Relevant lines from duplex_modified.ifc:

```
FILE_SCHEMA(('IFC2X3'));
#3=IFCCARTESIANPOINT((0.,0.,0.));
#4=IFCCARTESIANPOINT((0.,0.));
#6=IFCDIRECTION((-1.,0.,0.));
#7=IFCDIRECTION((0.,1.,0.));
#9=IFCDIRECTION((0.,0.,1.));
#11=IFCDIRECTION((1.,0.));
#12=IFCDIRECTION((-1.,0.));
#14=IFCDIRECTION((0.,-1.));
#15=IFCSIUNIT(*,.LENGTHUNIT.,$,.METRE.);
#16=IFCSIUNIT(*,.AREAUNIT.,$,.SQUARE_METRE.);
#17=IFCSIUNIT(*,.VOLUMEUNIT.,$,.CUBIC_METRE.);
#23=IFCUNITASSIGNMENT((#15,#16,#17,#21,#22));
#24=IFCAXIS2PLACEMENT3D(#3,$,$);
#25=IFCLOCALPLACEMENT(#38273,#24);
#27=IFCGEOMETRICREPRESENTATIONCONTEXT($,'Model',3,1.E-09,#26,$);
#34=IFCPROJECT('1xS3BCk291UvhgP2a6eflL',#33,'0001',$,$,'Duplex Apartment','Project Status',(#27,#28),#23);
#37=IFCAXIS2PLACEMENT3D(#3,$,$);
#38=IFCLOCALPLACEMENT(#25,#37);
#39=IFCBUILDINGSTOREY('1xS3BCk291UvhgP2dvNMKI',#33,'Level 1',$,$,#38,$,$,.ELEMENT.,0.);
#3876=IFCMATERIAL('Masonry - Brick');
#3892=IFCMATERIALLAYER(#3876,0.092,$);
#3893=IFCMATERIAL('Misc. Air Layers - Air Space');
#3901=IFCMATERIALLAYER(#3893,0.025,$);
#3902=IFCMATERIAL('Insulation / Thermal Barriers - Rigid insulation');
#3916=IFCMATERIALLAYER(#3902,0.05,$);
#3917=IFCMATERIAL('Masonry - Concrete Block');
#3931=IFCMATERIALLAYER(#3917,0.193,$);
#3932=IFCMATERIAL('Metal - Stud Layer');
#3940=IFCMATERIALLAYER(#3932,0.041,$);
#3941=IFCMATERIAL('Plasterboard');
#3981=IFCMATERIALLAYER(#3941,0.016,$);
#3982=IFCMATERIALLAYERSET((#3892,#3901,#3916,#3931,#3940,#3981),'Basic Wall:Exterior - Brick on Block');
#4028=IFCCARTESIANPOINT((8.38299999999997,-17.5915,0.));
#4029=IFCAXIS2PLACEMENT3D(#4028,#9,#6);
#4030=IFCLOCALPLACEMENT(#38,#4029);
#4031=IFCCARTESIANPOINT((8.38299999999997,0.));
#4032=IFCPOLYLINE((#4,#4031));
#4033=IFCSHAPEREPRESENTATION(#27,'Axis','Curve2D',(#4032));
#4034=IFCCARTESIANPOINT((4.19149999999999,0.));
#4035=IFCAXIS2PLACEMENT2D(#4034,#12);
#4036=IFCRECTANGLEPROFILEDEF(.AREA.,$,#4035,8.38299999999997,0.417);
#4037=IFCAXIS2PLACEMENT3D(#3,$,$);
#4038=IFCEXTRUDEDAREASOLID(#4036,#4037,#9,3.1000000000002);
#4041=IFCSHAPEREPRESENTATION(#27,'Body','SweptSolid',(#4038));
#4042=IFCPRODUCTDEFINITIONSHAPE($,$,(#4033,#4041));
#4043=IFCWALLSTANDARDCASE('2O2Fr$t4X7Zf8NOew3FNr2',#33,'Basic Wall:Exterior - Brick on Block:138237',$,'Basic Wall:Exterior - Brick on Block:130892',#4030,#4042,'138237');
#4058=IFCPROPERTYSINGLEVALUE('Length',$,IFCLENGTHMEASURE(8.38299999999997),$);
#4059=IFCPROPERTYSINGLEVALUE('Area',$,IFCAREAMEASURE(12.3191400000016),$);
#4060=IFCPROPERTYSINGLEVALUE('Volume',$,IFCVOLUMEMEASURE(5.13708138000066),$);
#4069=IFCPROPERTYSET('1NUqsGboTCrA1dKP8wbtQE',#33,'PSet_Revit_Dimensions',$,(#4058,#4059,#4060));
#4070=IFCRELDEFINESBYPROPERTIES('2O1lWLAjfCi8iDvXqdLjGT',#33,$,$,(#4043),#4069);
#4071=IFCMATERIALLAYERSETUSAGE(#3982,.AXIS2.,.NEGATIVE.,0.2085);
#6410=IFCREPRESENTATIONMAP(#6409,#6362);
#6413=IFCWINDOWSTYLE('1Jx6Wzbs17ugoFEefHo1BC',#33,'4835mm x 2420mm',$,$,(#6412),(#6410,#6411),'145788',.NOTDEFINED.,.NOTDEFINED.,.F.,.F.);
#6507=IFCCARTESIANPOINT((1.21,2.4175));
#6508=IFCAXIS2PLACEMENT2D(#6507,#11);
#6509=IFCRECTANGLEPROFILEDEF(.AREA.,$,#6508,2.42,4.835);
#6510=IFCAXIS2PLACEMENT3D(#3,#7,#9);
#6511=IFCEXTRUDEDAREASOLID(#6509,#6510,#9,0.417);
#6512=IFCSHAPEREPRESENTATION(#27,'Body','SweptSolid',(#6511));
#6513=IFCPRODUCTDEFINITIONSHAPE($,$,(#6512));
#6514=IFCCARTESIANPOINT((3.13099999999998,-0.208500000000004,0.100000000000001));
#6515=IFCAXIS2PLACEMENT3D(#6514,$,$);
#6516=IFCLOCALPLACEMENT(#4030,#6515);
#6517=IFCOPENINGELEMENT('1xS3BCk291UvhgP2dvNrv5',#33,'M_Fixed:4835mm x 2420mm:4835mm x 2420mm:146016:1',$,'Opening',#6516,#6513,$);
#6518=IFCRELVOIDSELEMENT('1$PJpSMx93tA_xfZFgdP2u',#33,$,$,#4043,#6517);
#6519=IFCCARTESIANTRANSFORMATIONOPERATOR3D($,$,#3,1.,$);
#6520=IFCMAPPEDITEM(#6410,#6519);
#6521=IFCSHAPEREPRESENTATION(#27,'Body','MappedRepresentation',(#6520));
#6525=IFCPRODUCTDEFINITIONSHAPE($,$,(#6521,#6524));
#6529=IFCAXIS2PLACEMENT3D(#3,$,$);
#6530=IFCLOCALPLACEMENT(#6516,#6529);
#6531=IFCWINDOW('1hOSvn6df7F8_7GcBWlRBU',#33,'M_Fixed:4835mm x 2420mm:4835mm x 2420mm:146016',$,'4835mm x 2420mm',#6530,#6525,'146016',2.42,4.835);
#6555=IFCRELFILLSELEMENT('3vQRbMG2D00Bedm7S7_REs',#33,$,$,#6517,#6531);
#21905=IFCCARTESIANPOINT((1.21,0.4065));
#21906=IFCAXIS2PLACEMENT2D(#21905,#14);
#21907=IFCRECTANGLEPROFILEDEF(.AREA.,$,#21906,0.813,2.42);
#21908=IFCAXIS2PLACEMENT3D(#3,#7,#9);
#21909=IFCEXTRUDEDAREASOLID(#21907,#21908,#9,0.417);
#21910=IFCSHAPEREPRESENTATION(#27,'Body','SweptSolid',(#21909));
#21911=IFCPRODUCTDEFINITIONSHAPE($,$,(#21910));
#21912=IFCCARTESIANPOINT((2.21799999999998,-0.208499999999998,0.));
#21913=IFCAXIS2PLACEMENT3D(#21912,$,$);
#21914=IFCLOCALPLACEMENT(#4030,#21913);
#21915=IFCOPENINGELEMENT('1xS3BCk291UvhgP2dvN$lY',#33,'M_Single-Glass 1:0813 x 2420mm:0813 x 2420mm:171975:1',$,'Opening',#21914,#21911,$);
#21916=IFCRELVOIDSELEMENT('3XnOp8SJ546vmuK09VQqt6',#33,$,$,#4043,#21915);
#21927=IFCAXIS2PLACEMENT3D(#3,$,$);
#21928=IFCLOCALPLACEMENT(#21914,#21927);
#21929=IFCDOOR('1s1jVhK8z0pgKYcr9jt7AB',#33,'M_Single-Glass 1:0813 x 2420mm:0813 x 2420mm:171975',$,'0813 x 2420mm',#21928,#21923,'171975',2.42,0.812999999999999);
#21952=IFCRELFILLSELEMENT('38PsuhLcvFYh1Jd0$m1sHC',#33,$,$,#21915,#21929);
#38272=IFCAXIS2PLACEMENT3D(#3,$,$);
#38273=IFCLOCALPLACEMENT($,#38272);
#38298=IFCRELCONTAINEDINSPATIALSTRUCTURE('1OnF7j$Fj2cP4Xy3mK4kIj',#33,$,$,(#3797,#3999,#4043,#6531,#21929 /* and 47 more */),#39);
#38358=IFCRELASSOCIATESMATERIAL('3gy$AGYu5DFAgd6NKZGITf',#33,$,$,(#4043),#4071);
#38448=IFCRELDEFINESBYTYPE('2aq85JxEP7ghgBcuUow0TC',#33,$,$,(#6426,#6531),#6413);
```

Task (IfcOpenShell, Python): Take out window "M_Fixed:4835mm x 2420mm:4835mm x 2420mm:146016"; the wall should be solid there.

```python
import ifcopenshell
import ifcopenshell.api.feature
import ifcopenshell.api.pset
import ifcopenshell.api.root
import ifcopenshell.geom
import ifcopenshell.util.element
import ifcopenshell.util.shape
import ifcopenshell.util.unit

model = ifcopenshell.open("duplex_modified.ifc")
area_scale = ifcopenshell.util.unit.calculate_unit_scale(model, "AREAUNIT")
volume_scale = ifcopenshell.util.unit.calculate_unit_scale(model, "VOLUMEUNIT")
settings = ifcopenshell.geom.settings()


def volume(element):
    """Net volume in cubic metres, openings subtracted."""
    shape = ifcopenshell.geom.create_shape(settings, element)
    return ifcopenshell.util.shape.get_volume(shape.geometry)


window = model.by_guid("1hOSvn6df7F8_7GcBWlRBU")
opening = window.FillsVoids[0].RelatingOpeningElement
wall = opening.VoidsElements[0].RelatingBuildingElement
before = volume(wall)

ifcopenshell.api.root.remove_product(model, product=window)
ifcopenshell.api.feature.remove_feature(model, feature=opening)

after = volume(wall)
thickness = 0.417  # wall thickness in metres

# Update the wall's stored quantities.
pset = model.by_id(ifcopenshell.util.element.get_pset(wall, "PSet_Revit_Dimensions", should_inherit=False)["id"])
ifcopenshell.api.pset.edit_pset(model, pset=pset, properties={
    "Area": model.create_entity("IfcAreaMeasure", after / thickness / area_scale),
    "Volume": model.create_entity("IfcVolumeMeasure", after / volume_scale),
})

print(f"wall volume {before:.3f} -> {after:.3f} m3")

model.write("duplex_modified_edited.ifc")
```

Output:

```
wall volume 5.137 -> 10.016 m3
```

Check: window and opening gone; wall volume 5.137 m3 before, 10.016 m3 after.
